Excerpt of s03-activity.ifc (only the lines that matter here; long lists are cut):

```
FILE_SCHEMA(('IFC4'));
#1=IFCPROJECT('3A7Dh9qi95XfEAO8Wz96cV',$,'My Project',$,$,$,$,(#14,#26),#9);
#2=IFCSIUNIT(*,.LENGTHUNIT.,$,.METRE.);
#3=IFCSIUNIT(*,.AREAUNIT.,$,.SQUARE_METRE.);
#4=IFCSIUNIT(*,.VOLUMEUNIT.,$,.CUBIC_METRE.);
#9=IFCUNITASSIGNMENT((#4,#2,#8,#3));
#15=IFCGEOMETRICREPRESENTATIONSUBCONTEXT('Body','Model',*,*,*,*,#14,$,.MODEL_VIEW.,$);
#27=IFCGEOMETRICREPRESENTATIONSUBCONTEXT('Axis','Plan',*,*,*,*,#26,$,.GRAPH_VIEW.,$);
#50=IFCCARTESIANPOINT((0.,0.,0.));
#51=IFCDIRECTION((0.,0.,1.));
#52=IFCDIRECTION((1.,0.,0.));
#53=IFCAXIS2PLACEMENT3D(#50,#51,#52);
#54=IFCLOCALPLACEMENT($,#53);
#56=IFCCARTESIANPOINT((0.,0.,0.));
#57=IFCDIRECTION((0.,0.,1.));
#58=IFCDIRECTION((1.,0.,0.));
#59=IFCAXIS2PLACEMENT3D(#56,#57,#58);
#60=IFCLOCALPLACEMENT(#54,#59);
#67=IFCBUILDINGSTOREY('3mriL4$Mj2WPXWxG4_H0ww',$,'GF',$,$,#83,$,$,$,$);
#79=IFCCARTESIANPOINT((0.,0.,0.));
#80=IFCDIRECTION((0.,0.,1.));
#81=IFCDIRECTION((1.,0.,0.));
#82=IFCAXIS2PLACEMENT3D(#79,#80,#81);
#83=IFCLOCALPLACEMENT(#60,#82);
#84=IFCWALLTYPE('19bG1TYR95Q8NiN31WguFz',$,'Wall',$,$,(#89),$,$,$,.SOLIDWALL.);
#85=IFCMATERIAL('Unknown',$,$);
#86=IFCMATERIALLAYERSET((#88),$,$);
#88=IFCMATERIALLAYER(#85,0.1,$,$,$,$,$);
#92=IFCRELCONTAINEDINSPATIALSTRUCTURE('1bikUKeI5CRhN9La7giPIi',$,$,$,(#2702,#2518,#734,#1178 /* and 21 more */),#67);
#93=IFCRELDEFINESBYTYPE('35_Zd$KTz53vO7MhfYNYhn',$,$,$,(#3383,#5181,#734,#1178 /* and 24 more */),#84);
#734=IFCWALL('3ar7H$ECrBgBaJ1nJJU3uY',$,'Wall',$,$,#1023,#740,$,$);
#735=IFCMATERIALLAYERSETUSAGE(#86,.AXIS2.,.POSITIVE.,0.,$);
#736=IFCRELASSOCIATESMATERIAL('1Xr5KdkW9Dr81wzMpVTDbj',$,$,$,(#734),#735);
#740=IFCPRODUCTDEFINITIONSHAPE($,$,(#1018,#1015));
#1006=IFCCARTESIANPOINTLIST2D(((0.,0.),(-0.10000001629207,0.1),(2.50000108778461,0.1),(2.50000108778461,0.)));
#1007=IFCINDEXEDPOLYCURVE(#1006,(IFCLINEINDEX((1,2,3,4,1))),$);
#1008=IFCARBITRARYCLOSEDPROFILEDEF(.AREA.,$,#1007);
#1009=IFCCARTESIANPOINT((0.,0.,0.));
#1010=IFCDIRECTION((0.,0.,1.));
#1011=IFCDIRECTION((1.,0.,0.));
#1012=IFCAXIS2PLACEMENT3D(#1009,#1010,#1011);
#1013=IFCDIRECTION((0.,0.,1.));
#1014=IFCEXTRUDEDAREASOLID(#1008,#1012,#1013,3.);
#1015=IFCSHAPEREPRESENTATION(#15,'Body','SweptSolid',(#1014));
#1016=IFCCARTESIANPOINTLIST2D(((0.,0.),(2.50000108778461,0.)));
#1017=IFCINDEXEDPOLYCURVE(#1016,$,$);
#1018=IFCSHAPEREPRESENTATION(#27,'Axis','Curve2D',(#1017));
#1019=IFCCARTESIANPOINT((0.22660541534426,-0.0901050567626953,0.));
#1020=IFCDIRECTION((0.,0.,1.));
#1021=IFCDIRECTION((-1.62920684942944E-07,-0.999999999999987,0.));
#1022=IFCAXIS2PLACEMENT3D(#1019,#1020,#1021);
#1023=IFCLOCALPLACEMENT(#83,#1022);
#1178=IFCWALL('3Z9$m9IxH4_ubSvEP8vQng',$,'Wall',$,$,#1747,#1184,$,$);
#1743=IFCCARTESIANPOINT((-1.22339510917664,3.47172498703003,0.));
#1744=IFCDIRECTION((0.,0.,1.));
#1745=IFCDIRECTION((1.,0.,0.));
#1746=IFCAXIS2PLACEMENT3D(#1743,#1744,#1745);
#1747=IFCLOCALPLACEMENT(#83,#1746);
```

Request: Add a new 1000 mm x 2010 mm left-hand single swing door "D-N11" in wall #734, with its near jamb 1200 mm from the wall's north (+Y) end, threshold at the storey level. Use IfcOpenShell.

```python
import numpy as np
import ifcopenshell
import ifcopenshell.api.feature
import ifcopenshell.api.geometry
import ifcopenshell.api.root
import ifcopenshell.api.spatial
import ifcopenshell.geom
import ifcopenshell.util.element
import ifcopenshell.util.placement
import ifcopenshell.util.representation
import ifcopenshell.util.shape
import ifcopenshell.util.unit

model = ifcopenshell.open("s03-activity.ifc")
unit_scale = ifcopenshell.util.unit.calculate_unit_scale(model)
settings = ifcopenshell.geom.settings()


def volume(element):
    """Net volume in cubic metres, openings subtracted."""
    shape = ifcopenshell.geom.create_shape(settings, element)
    return ifcopenshell.util.shape.get_volume(shape.geometry)


wall = model.by_guid("3ar7H$ECrBgBaJ1nJJU3uY")
storey = ifcopenshell.util.element.get_container(wall, ifc_class="IfcBuildingStorey")
context = ifcopenshell.util.representation.get_context(model, "Model", "Body", "MODEL_VIEW")
before = volume(wall)

width, height, from_end, sill = 1, 2.01, 1.2, 0.0  # metres

# The wall runs along its own X axis, and the end named is its -X end.
wall_shape = ifcopenshell.geom.create_shape(settings, wall)
x, y, z = ifcopenshell.util.shape.get_vertices(wall_shape.geometry).T
start = x.min() + from_end
face, thickness = float(y.min()), float(y.max() - y.min())
wall_matrix = ifcopenshell.util.placement.get_local_placement(wall.ObjectPlacement)
level = ifcopenshell.util.placement.get_local_placement(storey.ObjectPlacement)[2, 3]


def in_wall(x, y):
    """Placement at x, y metres in the wall's axes, at sill height."""
    matrix = wall_matrix.copy()
    matrix[:, 3] = wall_matrix @ np.array([x / unit_scale, y / unit_scale, 0.0, 1.0])
    matrix[2, 3] = level + sill / unit_scale
    return matrix


# Opening: a box that overshoots both wall faces by 50 mm.
opening = ifcopenshell.api.root.create_entity(model, ifc_class="IfcOpeningElement", predefined_type="OPENING")
box = ifcopenshell.api.geometry.add_wall_representation(
    model, context=context, length=width, height=height, thickness=thickness + 0.1
)
ifcopenshell.api.geometry.assign_representation(model, product=opening, representation=box)
ifcopenshell.api.geometry.edit_object_placement(model, product=opening, matrix=in_wall(start, face - 0.05), is_si=False)
ifcopenshell.api.feature.add_feature(model, feature=opening, element=wall)

door = ifcopenshell.api.root.create_entity(model, ifc_class="IfcDoor", name="D-N11", predefined_type="DOOR")
door.OverallWidth, door.OverallHeight = width / unit_scale, height / unit_scale
door.OperationType = "SINGLE_SWING_LEFT"
body = ifcopenshell.api.geometry.add_door_representation(
    model,
    context=context,
    overall_width=door.OverallWidth,
    overall_height=door.OverallHeight,
    operation_type="SINGLE_SWING_LEFT",
    lining_properties={"LiningDepth": thickness / unit_scale, "ThresholdDepth": thickness / unit_scale},
)
ifcopenshell.api.geometry.assign_representation(model, product=door, representation=body)
ifcopenshell.api.spatial.assign_container(model, products=[door], relating_structure=storey)
ifcopenshell.api.feature.add_filling(model, opening=opening, element=door)

# The lining spans the wall, so the door starts at the wall face.
ifcopenshell.api.geometry.edit_object_placement(model, product=door, matrix=in_wall(start, face), is_si=False)

after = volume(wall)

print(f"wall volume {before:.3f} -> {after:.3f} m3")

model.write("s03-activity-out.ifc")
```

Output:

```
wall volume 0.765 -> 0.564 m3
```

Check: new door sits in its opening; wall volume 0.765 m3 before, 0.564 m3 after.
